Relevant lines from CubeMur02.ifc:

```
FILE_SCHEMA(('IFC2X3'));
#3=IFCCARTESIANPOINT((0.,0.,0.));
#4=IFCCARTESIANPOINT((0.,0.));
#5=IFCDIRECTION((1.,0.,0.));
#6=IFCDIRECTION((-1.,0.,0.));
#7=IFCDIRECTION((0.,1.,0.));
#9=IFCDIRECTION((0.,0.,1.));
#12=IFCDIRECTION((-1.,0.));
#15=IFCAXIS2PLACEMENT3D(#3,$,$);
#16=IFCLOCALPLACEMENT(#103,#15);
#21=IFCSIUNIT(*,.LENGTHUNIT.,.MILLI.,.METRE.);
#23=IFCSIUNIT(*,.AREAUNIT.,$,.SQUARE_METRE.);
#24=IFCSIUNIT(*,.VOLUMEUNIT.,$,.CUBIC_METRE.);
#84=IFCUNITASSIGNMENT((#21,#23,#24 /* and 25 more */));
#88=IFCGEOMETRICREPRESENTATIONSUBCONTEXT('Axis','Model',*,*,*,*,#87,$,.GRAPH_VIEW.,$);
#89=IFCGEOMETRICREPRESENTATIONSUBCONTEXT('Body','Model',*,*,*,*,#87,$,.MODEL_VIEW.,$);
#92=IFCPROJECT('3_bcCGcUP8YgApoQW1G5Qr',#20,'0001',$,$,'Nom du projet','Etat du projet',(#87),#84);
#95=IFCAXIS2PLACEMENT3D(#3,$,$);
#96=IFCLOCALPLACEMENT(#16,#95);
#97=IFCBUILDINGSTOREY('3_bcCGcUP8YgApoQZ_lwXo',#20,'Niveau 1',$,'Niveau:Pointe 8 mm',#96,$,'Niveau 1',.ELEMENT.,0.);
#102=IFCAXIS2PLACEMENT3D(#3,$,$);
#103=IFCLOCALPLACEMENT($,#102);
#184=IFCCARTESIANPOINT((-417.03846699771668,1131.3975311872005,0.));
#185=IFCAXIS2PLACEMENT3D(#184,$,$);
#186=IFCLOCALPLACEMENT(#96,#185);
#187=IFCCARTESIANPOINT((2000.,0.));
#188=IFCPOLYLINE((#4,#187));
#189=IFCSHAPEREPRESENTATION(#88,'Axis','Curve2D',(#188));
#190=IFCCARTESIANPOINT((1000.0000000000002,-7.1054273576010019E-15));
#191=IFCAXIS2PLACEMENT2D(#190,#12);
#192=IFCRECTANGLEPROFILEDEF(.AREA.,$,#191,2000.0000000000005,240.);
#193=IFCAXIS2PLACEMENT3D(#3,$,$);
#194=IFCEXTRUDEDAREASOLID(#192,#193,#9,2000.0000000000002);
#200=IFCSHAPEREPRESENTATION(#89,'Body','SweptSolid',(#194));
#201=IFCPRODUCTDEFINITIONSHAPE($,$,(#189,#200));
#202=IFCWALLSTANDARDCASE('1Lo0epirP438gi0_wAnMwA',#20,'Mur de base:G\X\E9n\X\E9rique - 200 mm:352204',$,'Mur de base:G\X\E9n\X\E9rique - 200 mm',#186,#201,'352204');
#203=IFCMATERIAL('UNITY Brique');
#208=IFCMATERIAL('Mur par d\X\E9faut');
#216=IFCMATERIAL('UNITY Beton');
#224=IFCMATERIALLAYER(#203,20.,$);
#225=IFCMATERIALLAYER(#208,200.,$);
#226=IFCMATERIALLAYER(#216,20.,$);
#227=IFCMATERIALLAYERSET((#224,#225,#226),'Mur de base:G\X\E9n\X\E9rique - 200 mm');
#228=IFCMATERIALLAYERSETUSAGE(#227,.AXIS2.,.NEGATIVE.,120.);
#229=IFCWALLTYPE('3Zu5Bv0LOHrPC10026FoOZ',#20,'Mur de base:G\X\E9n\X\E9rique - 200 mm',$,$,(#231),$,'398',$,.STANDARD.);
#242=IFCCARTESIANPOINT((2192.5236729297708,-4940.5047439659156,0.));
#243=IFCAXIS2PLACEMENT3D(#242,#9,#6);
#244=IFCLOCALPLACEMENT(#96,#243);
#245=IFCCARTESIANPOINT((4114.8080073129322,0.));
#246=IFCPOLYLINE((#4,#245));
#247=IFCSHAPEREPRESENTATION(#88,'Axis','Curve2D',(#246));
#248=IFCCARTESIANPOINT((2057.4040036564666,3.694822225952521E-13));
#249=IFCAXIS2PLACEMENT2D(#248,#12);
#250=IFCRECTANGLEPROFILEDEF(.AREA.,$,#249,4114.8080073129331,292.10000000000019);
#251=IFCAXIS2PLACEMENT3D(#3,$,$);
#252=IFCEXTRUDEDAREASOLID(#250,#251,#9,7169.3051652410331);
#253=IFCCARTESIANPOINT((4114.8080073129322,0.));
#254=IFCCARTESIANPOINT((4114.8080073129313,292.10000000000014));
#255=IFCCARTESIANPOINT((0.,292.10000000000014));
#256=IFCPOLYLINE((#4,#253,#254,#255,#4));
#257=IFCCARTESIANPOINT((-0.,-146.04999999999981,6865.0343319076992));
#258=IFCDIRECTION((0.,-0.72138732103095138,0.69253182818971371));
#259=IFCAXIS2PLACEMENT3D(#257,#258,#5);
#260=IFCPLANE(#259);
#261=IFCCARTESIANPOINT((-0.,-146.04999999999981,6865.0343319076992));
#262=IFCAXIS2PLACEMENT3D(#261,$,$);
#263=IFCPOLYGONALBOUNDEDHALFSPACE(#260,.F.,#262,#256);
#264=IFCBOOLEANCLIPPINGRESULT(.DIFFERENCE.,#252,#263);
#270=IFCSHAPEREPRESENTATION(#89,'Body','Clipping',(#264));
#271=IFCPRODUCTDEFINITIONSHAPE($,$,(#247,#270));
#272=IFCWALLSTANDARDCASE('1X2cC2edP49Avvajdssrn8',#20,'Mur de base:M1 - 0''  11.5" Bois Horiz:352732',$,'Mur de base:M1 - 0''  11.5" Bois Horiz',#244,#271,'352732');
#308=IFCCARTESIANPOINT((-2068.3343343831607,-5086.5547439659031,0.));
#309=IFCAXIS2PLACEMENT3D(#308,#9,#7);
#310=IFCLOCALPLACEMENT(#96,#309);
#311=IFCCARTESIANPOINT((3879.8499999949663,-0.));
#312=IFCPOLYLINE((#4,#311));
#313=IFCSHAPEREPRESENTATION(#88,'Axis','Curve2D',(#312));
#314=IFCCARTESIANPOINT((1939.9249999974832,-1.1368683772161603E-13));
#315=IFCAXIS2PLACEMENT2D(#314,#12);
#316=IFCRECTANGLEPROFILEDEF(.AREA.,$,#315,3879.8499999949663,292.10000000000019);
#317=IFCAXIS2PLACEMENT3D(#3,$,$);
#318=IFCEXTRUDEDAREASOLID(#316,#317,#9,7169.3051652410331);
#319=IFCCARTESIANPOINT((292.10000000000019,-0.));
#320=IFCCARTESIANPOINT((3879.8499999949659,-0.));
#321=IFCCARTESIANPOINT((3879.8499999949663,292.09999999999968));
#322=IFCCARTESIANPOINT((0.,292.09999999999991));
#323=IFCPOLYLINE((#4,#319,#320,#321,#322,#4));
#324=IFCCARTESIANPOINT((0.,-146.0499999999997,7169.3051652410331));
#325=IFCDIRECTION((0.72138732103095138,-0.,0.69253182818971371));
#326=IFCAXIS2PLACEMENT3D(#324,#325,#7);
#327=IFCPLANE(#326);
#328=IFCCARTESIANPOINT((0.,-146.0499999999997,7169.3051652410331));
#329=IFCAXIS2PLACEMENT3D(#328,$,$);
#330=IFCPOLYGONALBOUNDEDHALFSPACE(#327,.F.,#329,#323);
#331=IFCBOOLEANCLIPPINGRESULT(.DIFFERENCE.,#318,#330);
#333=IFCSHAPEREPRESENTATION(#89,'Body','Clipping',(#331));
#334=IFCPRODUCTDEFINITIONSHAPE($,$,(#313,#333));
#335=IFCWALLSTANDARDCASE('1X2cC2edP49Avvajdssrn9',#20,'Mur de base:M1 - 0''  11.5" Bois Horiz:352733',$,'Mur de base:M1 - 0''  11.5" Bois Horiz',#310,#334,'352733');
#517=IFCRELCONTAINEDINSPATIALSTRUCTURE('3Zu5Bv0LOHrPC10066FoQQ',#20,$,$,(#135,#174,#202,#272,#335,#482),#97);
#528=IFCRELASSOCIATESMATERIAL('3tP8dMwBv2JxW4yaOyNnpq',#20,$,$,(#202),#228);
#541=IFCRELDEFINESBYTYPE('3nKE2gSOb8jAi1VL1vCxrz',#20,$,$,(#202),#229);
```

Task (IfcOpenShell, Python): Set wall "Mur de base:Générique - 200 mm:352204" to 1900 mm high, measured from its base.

```python
import ifcopenshell
import ifcopenshell.geom
import ifcopenshell.util.representation
import ifcopenshell.util.shape

model = ifcopenshell.open("CubeMur02.ifc")
settings = ifcopenshell.geom.settings()


def volume(element):
    """Net volume in cubic metres, openings subtracted."""
    shape = ifcopenshell.geom.create_shape(settings, element)
    return ifcopenshell.util.shape.get_volume(shape.geometry)


wall = model.by_id(202)
before = volume(wall)

body = ifcopenshell.util.representation.get_representation(wall, "Model", "Body")
solid = body.Items[0]
old_height = solid.Depth
solid.Depth = 1900.0
after = volume(wall)

print(f"height {old_height:g} -> {solid.Depth:g}, volume {before:.3f} -> {after:.3f} m3")

model.write("CubeMur02_v2.ifc")
```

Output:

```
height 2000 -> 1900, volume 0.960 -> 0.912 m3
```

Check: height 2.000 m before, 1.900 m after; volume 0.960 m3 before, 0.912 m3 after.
